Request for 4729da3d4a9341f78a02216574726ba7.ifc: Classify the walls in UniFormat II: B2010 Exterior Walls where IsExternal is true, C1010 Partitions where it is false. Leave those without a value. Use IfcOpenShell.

First a look at what the model holds.

```python
import ifcopenshell
import ifcopenshell.util.element

model = ifcopenshell.open("4729da3d4a9341f78a02216574726ba7.ifc")
print(model.schema)
print("classifications:", [c.Name for c in model.by_type("IfcClassification")])
values = [ifcopenshell.util.element.get_pset(e, "Pset_WallCommon", "IsExternal") for e in model.by_type("IfcWall")]
for value in (True, False, None):
    print("IsExternal", value, values.count(value))
```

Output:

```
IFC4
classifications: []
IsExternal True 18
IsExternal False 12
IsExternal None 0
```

```python
import ifcopenshell
import ifcopenshell.api.classification
import ifcopenshell.util.element

model = ifcopenshell.open("4729da3d4a9341f78a02216574726ba7.ifc")

system = ifcopenshell.api.classification.add_classification(model, classification="UniFormat II")

walls = model.by_type("IfcWall")
external = {e: ifcopenshell.util.element.get_pset(e, "Pset_WallCommon", "IsExternal") for e in walls}
for flag, code, name in ((True, "B2010", "Exterior Walls"), (False, "C1010", "Partitions")):
    products = [e for e in walls if external[e] is flag]
    ifcopenshell.api.classification.add_reference(
        model, products=products, classification=system, identification=code, name=name
    )
    print(code, len(products))

model.write("4729da3d4a9341f78a02216574726ba7_rev.ifc")
```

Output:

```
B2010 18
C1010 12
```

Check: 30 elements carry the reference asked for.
